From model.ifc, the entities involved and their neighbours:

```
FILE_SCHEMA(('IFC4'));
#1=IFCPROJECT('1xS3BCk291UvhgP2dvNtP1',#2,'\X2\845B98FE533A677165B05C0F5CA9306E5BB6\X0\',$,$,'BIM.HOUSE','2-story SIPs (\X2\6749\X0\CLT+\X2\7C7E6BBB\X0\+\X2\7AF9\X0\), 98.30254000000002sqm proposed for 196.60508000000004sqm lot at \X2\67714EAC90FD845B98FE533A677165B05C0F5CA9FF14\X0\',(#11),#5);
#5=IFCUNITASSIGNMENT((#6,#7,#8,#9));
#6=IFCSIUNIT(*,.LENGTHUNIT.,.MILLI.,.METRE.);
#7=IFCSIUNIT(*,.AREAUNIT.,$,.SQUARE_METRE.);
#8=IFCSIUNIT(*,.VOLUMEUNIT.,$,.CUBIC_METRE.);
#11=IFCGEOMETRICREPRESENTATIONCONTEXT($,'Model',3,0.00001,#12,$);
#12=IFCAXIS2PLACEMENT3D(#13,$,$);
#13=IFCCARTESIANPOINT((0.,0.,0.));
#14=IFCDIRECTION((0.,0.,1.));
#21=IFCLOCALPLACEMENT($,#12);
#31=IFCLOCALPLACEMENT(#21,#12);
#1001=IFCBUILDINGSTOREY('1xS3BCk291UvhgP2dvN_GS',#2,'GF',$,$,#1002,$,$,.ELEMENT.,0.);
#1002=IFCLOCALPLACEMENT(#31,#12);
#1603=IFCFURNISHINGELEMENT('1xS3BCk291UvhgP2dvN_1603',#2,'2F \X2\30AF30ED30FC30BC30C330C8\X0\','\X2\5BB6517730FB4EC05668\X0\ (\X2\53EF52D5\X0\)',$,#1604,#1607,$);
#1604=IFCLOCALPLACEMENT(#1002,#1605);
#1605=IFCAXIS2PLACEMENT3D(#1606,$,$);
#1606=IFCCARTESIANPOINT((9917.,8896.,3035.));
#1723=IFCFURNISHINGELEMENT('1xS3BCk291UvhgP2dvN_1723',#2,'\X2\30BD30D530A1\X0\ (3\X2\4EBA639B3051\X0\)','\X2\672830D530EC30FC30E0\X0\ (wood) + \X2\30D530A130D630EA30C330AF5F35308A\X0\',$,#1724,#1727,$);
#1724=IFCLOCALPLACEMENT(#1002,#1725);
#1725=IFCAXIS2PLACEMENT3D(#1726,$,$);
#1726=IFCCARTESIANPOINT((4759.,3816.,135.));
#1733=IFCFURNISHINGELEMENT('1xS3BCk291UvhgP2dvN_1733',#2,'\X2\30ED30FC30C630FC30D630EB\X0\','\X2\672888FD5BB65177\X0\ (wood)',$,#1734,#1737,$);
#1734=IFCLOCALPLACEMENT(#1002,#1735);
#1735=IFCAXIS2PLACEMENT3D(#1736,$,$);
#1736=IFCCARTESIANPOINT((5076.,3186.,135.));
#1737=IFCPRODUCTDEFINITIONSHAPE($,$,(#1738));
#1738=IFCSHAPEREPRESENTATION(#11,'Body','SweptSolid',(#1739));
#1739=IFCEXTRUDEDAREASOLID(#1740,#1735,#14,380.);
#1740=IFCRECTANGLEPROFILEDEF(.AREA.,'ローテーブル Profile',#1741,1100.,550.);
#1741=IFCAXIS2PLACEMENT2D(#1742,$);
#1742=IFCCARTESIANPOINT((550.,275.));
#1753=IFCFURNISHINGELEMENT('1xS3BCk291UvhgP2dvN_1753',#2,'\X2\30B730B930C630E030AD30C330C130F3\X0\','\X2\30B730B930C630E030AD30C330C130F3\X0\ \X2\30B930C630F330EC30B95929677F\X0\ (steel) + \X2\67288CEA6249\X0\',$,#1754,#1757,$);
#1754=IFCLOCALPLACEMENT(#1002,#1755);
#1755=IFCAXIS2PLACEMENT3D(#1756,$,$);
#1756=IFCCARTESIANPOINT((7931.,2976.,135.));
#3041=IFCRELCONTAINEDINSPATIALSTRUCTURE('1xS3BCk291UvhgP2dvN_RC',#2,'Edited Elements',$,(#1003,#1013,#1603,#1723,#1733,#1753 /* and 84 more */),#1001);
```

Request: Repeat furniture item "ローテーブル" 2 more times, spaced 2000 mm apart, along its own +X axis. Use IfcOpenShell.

```python
import ifcopenshell
import ifcopenshell.api.geometry
import ifcopenshell.api.root
import ifcopenshell.util.element
import ifcopenshell.util.placement
import ifcopenshell.util.unit

model = ifcopenshell.open("model.ifc")
unit_scale = ifcopenshell.util.unit.calculate_unit_scale(model)


def reuse_history(source, copy):
    """copy_class also copies each property set's owner history, people and application; keep the originals."""
    for rel in copy.IsDefinedBy:
        if rel.is_a("IfcRelDefinesByProperties") and (history := rel.RelatingPropertyDefinition.OwnerHistory):
            rel.RelatingPropertyDefinition.OwnerHistory = source.OwnerHistory
            ifcopenshell.util.element.remove_deep2(model, history)


source = model.by_guid("1xS3BCk291UvhgP2dvN_1733")
base = ifcopenshell.util.placement.get_local_placement(source.ObjectPlacement)
step = base[:3, 0] * 2 / unit_scale

for i in range(1, 3):
    copy = ifcopenshell.api.root.copy_class(model, product=source)
    copy.Representation = ifcopenshell.util.element.copy_deep(
        model, source.Representation, exclude=["IfcGeometricRepresentationContext", "IfcRepresentationMap"]
    )
    reuse_history(source, copy)
    matrix = base.copy()
    matrix[:3, 3] += i * step
    print("added at", matrix[:3, 3].round(3) + 0.0)
    ifcopenshell.api.geometry.edit_object_placement(model, product=copy, matrix=matrix, is_si=False)

model.write("model-out.ifc")
```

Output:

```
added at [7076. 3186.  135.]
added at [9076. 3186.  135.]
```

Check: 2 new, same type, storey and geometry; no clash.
